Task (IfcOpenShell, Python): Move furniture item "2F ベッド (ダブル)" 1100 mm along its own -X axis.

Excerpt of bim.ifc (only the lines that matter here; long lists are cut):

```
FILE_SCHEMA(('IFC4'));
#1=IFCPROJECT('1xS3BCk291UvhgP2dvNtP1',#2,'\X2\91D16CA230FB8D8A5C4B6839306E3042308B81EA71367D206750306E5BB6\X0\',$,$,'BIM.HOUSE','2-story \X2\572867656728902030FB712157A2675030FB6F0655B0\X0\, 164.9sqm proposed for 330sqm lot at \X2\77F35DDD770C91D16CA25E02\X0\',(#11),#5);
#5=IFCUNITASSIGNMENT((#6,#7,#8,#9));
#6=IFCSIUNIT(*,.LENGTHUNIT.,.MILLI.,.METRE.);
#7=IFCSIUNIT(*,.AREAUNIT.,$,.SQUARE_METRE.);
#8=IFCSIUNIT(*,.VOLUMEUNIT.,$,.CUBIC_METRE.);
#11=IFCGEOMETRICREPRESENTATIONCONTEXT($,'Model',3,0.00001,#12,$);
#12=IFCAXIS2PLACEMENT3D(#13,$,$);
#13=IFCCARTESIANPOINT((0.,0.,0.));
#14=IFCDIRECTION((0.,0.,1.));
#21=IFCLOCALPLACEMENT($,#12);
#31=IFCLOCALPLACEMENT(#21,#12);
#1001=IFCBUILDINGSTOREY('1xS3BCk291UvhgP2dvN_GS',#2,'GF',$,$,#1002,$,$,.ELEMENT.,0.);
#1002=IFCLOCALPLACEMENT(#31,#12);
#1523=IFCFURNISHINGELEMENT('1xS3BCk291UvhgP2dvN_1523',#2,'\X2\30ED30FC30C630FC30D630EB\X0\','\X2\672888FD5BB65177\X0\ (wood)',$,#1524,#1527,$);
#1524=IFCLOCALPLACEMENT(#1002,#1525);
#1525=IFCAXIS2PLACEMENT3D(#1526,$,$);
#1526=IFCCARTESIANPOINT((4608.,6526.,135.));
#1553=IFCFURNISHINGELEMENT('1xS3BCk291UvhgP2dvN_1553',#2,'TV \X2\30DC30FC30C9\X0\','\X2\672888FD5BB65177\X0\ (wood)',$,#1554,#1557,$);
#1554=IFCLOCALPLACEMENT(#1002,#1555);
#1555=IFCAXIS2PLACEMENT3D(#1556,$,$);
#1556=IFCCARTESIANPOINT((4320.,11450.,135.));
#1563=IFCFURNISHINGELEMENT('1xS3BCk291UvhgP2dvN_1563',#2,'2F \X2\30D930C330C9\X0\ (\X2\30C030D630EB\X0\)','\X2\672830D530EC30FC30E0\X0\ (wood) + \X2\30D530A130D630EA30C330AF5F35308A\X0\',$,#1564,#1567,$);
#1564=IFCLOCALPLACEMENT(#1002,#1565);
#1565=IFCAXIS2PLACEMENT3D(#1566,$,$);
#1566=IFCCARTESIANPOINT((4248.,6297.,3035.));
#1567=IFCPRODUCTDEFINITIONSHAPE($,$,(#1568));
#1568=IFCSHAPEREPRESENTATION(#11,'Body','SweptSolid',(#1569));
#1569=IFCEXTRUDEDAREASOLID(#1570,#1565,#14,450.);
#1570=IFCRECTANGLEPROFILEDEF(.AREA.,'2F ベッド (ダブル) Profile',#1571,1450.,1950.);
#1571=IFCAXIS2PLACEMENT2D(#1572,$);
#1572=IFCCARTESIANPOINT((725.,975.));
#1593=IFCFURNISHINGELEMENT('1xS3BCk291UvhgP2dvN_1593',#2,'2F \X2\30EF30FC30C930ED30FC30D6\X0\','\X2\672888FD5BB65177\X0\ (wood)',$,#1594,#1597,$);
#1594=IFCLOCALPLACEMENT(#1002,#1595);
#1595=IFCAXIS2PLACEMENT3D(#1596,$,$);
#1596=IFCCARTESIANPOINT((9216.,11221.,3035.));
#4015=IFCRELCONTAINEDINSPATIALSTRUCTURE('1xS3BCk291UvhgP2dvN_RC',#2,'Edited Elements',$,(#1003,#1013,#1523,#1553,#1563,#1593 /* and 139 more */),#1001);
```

```python
import ifcopenshell
import ifcopenshell.api.geometry
import ifcopenshell.util.placement
import ifcopenshell.util.unit

model = ifcopenshell.open("bim.ifc")
unit_scale = ifcopenshell.util.unit.calculate_unit_scale(model)

item = model.by_id(1563)
matrix = ifcopenshell.util.placement.get_local_placement(item.ObjectPlacement)
matrix[:3, 3] -= matrix[:3, 0] * 1.1 / unit_scale
ifcopenshell.api.geometry.edit_object_placement(model, product=item, matrix=matrix, is_si=False)

print(ifcopenshell.util.placement.get_local_placement(item.ObjectPlacement).round(3) + 0.0)

model.write("bim_updated.ifc")
```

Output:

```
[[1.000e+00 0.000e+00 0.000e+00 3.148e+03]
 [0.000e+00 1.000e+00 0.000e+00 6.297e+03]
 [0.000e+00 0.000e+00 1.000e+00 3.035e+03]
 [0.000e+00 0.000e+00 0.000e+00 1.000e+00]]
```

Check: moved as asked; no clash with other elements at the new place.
